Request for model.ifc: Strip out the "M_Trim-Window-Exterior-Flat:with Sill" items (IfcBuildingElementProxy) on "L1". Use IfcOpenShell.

First a look at what the model holds.

```python
import ifcopenshell
import ifcopenshell.util.element

model = ifcopenshell.open("model.ifc")
print(model.schema)
storey = next(s for s in model.by_type("IfcBuildingStorey") if s.Name == "L1")
proxies = [e for e in ifcopenshell.util.element.get_decomposition(storey) if e.is_a("IfcBuildingElementProxy")]
seen = {}
for e in proxies:
    element_type = ifcopenshell.util.element.get_type(e)
    name = element_type.Name if element_type not in (None, e) else None
    seen[name] = seen.get(name, 0) + 1
for name, count in sorted(seen.items(), key=str):
    print(count, "x", name)
```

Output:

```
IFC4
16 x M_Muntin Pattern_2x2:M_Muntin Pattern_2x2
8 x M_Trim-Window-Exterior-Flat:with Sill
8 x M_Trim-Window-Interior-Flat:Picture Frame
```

```python
import ifcopenshell
import ifcopenshell.api.root
import ifcopenshell.util.element

model = ifcopenshell.open("model.ifc")

storey = next(s for s in model.by_type("IfcBuildingStorey") if s.Name == "L1")
proxies = [e for e in ifcopenshell.util.element.get_decomposition(storey) if e.is_a("IfcBuildingElementProxy")]
targets = [e for e in proxies if (t := ifcopenshell.util.element.get_type(e)) not in (None, e) and t.Name == "M_Trim-Window-Exterior-Flat:with Sill"]

for e in targets:
    ifcopenshell.api.root.remove_product(model, product=e)
print(len(targets), "removed")

model.write("model-out.ifc")
```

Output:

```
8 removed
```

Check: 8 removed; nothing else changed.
